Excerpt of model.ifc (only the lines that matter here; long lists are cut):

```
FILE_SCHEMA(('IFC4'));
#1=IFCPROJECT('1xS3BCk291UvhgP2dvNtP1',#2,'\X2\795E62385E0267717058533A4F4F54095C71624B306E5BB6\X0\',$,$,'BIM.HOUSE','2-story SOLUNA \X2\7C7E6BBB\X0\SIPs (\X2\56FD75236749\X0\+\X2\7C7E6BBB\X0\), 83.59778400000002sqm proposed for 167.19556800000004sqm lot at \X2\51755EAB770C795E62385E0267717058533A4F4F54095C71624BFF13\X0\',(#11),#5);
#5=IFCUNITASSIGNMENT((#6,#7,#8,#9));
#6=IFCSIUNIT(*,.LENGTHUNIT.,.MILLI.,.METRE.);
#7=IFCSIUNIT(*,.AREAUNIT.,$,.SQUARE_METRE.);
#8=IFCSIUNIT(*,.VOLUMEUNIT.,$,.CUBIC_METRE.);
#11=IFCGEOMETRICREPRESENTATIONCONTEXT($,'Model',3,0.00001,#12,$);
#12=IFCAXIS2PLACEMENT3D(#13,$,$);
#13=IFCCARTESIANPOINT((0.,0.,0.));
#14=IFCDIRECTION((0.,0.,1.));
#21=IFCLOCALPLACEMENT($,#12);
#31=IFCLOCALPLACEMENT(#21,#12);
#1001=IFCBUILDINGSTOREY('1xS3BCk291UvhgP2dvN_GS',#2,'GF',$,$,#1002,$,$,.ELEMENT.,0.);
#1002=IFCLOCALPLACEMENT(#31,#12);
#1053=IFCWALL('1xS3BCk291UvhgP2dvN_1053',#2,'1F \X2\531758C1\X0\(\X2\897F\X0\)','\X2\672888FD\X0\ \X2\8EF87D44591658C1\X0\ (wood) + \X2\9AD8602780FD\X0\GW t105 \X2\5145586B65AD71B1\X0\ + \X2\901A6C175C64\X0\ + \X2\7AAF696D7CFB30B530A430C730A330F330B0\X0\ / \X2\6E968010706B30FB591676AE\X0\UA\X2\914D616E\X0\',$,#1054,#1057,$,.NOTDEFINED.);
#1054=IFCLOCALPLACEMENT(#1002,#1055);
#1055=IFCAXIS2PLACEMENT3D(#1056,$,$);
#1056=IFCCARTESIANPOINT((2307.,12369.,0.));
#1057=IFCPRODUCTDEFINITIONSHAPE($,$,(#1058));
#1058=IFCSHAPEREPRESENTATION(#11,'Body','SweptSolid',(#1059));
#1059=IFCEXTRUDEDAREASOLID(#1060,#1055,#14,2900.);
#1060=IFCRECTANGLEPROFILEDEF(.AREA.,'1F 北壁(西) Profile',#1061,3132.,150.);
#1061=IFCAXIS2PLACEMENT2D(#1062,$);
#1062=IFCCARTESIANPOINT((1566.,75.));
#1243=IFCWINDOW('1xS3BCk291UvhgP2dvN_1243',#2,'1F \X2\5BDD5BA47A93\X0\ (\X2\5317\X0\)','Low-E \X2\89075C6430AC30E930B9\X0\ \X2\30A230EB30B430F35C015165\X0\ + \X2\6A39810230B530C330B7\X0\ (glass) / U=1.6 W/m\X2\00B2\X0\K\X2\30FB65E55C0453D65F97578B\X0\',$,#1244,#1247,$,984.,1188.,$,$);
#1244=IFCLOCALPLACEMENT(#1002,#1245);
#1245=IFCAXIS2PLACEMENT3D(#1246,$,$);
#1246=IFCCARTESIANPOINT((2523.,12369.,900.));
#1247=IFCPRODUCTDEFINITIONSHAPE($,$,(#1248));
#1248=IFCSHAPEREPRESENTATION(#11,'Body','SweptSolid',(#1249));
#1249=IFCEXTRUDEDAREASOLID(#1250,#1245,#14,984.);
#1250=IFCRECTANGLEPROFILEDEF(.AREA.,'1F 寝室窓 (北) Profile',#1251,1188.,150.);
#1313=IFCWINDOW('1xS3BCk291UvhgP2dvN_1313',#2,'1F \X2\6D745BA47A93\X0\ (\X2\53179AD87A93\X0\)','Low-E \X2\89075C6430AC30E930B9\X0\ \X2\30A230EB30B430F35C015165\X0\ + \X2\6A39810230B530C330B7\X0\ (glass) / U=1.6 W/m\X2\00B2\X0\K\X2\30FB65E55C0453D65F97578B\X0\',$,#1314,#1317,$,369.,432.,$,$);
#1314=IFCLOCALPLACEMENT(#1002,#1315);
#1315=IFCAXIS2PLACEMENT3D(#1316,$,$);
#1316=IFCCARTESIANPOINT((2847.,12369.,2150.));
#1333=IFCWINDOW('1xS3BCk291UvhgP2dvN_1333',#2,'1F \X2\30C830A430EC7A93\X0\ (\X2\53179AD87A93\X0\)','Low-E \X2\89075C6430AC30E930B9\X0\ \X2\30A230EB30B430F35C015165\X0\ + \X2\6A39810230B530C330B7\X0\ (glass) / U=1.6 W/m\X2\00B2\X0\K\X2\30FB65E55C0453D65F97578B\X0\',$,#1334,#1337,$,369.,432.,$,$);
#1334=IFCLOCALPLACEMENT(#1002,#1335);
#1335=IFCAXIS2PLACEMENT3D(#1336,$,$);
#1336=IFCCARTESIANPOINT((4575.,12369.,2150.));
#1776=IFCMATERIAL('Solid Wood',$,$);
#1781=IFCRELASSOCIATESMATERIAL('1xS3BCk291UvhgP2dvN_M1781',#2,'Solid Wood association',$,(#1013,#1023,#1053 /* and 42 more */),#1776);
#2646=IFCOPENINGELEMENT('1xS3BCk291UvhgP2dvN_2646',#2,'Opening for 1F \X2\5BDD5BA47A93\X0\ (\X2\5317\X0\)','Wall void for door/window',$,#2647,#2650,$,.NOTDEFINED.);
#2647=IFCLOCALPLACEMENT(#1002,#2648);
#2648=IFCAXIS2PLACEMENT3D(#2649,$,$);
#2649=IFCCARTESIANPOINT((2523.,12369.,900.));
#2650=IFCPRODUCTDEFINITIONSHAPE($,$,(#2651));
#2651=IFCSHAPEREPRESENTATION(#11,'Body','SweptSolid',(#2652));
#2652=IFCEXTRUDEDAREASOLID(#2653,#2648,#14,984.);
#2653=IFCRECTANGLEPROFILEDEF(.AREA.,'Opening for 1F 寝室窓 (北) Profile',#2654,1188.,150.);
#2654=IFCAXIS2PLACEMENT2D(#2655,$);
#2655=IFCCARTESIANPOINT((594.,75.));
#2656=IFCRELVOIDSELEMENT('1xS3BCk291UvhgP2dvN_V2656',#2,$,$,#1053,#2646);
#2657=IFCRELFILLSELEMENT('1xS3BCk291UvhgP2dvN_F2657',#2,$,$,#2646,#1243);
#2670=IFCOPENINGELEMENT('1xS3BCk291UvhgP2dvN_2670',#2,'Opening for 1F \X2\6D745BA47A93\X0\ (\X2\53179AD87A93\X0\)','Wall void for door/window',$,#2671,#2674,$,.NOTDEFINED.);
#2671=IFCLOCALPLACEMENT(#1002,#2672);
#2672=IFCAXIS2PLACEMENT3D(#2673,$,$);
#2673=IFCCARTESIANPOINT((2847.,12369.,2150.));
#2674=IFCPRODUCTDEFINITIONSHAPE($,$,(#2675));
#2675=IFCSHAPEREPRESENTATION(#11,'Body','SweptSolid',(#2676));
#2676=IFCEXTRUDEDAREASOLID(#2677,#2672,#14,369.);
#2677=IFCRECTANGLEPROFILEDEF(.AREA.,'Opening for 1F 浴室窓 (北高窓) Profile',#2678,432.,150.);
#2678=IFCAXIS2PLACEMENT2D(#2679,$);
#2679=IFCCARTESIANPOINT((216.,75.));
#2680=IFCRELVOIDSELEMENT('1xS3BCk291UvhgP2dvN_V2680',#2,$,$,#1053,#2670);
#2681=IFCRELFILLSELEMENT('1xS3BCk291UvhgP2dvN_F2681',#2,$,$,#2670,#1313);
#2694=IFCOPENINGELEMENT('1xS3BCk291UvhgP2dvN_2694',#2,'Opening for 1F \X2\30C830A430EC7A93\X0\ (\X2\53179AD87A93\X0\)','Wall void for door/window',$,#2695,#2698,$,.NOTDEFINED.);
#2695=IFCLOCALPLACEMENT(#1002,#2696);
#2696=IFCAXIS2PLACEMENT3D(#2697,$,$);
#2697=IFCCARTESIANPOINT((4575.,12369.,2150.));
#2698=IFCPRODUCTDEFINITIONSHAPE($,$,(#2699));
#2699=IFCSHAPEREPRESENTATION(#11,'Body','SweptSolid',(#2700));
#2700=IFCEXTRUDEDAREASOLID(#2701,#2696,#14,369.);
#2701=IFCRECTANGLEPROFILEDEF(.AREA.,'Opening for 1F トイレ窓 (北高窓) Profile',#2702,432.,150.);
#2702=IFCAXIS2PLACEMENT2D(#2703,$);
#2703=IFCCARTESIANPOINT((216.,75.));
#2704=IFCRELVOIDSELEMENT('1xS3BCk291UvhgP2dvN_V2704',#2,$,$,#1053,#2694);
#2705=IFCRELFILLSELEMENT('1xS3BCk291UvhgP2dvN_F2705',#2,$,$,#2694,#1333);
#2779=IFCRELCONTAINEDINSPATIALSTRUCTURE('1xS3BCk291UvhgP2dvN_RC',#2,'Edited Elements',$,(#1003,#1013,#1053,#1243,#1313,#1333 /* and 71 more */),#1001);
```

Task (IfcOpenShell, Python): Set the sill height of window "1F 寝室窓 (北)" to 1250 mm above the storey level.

```python
import numpy as np
import ifcopenshell
import ifcopenshell.api.geometry
import ifcopenshell.geom
import ifcopenshell.util.element
import ifcopenshell.util.placement
import ifcopenshell.util.shape
import ifcopenshell.util.unit

model = ifcopenshell.open("model.ifc")
unit_scale = ifcopenshell.util.unit.calculate_unit_scale(model)

window = model.by_guid("1xS3BCk291UvhgP2dvN_1243")
opening = window.FillsVoids[0].RelatingOpeningElement
storey = ifcopenshell.util.element.get_container(window, ifc_class="IfcBuildingStorey")
level = ifcopenshell.util.placement.get_local_placement(storey.ObjectPlacement)[2, 3]

# The opening's origin need not be at the sill, so measure its lowest point.
shape = ifcopenshell.geom.create_shape(ifcopenshell.geom.settings(), opening)
bottom = ifcopenshell.util.shape.get_shape_bottom_elevation(shape, shape.geometry) / unit_scale
dz = level + 1250.0 - bottom

shift = np.array([0.0, 0.0, dz])
# The window is not placed relative to its opening, so move both.
for product in (opening, window):
    matrix = ifcopenshell.util.placement.get_local_placement(product.ObjectPlacement)
    matrix[:3, 3] += shift
    ifcopenshell.api.geometry.edit_object_placement(model, product=product, matrix=matrix, is_si=False)

print(f"moved by {dz * unit_scale:+.3f} m")

model.write("model-out.ifc")
```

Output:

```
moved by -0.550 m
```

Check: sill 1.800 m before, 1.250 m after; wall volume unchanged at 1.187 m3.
